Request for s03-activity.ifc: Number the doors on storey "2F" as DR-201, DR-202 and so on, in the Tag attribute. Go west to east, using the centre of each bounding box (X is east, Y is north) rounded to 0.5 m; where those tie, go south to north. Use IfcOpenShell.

First a look at what the model holds.

```python
import ifcopenshell
import ifcopenshell.util.element
import ifcopenshell.util.placement

model = ifcopenshell.open("s03-activity.ifc")
print(model.schema)
storey = next(s for s in model.by_type("IfcBuildingStorey") if s.Name == "2F")
doors = [e for e in ifcopenshell.util.element.get_decomposition(storey) if e.is_a("IfcDoor")]
for e in sorted(doors, key=lambda e: e.id()):
    origin = ifcopenshell.util.placement.get_local_placement(e.ObjectPlacement)[:3, 3]
    print(e.id(), e.Tag, e.Name, origin.round(2) + 0.0, sep=" | ")
```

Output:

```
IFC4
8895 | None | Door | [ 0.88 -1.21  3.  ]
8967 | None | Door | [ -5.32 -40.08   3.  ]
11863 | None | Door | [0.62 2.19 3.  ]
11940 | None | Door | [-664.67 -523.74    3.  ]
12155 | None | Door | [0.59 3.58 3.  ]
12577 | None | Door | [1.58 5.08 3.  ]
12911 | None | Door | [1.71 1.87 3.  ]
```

```python
import ifcopenshell
import ifcopenshell.geom
import ifcopenshell.util.element
import ifcopenshell.util.shape

model = ifcopenshell.open("s03-activity.ifc")
settings = ifcopenshell.geom.settings()
settings.set("use-world-coords", True)


def centre(element):
    shape = ifcopenshell.geom.create_shape(settings, element)
    return ifcopenshell.util.shape.get_bbox_centroid(shape.geometry)


storey = next(s for s in model.by_type("IfcBuildingStorey") if s.Name == "2F")
doors = [e for e in ifcopenshell.util.element.get_decomposition(storey) if e.is_a("IfcDoor")]

# Insertion points can sit at a corner or the storey origin, so sort by the geometry (in metres).
centres = {e: centre(e) for e in doors}
doors.sort(key=lambda e: (round(centres[e][0] / 0.5), centres[e][1]))

for i, e in enumerate(doors, start=1):
    number = f"DR-2{i:02d}"
    e.Tag = number
    print(e.id(), number)

model.write("s03-activity_edited.ifc")
```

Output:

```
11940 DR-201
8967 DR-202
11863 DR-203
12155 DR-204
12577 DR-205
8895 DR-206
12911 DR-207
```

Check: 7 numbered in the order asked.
